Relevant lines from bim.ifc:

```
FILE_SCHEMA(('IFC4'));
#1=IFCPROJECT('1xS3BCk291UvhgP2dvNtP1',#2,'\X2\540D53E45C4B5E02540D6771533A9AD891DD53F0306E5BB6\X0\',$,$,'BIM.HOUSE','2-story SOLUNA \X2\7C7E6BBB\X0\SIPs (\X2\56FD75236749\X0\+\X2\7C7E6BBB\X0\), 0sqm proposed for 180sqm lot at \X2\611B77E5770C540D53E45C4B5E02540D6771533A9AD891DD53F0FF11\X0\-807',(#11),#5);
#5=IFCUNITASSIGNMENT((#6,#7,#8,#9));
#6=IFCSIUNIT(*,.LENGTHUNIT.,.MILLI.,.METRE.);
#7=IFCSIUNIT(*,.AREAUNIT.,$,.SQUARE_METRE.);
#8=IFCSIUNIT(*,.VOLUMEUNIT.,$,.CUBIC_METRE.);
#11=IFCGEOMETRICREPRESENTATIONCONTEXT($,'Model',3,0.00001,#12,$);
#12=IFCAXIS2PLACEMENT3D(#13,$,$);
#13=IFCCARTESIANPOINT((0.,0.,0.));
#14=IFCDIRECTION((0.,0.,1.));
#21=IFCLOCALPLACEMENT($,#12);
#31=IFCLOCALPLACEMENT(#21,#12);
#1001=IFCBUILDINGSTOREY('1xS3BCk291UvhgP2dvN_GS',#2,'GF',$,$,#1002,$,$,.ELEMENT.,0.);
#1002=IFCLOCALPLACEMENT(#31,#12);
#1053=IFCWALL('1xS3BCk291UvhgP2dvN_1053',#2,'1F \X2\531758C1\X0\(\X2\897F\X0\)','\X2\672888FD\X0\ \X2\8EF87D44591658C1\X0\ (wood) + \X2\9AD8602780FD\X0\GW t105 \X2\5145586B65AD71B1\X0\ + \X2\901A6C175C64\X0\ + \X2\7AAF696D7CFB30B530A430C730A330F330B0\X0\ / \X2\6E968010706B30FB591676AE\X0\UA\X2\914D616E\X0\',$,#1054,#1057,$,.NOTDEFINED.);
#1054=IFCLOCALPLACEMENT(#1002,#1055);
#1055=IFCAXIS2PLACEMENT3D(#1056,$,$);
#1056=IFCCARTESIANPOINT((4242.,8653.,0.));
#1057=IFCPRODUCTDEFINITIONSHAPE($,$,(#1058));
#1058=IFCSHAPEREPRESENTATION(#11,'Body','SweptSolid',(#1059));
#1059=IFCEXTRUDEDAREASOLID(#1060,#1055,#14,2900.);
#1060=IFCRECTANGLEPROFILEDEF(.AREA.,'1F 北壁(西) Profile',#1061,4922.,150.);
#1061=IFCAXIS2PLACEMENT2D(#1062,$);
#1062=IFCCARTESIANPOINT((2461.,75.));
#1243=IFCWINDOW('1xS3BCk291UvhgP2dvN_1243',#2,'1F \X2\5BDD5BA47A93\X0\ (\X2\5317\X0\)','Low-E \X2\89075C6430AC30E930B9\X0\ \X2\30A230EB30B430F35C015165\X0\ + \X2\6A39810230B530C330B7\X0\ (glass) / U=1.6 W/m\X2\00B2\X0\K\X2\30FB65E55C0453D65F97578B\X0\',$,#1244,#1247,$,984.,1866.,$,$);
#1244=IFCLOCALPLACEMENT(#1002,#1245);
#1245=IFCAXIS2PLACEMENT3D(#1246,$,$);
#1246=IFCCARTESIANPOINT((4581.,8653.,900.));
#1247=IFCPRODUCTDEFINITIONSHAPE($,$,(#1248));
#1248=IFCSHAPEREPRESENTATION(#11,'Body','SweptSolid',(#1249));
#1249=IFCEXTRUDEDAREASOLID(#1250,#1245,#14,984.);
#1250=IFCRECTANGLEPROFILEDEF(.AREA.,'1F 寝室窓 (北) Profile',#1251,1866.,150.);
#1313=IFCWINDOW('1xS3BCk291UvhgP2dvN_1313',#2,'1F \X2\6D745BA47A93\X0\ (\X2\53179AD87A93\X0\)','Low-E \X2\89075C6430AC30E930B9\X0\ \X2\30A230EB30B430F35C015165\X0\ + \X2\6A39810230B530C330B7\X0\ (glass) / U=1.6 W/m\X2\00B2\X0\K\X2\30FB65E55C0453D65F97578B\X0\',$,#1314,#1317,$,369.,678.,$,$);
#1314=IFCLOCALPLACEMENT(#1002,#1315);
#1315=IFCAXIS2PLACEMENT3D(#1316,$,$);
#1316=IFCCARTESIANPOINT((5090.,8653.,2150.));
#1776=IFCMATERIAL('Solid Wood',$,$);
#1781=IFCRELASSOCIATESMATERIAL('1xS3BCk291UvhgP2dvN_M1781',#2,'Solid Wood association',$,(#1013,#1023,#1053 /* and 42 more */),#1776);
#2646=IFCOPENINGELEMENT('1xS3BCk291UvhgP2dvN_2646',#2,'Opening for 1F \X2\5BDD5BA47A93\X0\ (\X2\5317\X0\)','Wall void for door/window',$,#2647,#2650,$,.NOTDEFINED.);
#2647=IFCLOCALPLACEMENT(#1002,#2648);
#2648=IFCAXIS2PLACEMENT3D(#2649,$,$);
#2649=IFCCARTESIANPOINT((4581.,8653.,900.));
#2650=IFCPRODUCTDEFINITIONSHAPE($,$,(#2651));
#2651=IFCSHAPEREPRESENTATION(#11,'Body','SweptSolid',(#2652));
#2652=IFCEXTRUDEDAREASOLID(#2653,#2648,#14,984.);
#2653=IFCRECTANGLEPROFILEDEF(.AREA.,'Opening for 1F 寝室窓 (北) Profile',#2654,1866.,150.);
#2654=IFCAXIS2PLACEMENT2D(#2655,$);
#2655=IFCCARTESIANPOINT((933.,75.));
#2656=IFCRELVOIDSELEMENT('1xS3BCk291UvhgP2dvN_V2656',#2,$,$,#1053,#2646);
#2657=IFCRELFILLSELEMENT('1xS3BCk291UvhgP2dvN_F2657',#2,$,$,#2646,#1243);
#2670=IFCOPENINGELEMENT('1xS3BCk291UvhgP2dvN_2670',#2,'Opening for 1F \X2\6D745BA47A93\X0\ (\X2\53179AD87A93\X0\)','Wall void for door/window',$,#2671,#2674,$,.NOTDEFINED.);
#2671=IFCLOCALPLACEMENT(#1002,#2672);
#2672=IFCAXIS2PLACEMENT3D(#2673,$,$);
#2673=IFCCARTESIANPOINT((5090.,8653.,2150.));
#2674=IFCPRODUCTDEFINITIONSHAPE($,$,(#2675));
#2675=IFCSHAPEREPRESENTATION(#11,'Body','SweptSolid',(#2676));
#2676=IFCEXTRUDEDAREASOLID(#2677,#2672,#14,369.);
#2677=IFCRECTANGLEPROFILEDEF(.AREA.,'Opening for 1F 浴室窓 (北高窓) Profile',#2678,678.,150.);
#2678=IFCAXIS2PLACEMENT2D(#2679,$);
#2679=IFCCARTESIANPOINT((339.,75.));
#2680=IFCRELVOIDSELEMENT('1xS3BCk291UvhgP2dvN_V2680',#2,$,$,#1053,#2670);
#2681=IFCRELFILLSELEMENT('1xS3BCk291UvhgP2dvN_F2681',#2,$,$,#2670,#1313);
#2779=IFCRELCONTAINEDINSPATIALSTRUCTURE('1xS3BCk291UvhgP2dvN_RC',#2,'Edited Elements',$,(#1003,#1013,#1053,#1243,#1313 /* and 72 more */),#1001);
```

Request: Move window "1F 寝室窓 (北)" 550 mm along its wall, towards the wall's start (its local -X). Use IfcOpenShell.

```python
import ifcopenshell
import ifcopenshell.api.geometry
import ifcopenshell.util.placement
import ifcopenshell.util.unit

model = ifcopenshell.open("bim.ifc")
unit_scale = ifcopenshell.util.unit.calculate_unit_scale(model)

window = model.by_id(1243)
opening = window.FillsVoids[0].RelatingOpeningElement
wall = opening.VoidsElements[0].RelatingBuildingElement

wall_matrix = ifcopenshell.util.placement.get_local_placement(wall.ObjectPlacement)
shift = wall_matrix[:3, 0] * -0.55 / unit_scale
before = ifcopenshell.util.placement.get_local_placement(window.ObjectPlacement)[:3, 3].copy()

# The window is not placed relative to its opening, so move both.
for product in (opening, window):
    matrix = ifcopenshell.util.placement.get_local_placement(product.ObjectPlacement)
    matrix[:3, 3] += shift
    ifcopenshell.api.geometry.edit_object_placement(model, product=product, matrix=matrix, is_si=False)

after = ifcopenshell.util.placement.get_local_placement(window.ObjectPlacement)[:3, 3]
print("window moved by", (after - before).round(3) + 0.0)

model.write("bim-out.ifc")
```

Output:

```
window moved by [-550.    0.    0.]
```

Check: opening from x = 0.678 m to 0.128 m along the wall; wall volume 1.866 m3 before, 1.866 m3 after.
